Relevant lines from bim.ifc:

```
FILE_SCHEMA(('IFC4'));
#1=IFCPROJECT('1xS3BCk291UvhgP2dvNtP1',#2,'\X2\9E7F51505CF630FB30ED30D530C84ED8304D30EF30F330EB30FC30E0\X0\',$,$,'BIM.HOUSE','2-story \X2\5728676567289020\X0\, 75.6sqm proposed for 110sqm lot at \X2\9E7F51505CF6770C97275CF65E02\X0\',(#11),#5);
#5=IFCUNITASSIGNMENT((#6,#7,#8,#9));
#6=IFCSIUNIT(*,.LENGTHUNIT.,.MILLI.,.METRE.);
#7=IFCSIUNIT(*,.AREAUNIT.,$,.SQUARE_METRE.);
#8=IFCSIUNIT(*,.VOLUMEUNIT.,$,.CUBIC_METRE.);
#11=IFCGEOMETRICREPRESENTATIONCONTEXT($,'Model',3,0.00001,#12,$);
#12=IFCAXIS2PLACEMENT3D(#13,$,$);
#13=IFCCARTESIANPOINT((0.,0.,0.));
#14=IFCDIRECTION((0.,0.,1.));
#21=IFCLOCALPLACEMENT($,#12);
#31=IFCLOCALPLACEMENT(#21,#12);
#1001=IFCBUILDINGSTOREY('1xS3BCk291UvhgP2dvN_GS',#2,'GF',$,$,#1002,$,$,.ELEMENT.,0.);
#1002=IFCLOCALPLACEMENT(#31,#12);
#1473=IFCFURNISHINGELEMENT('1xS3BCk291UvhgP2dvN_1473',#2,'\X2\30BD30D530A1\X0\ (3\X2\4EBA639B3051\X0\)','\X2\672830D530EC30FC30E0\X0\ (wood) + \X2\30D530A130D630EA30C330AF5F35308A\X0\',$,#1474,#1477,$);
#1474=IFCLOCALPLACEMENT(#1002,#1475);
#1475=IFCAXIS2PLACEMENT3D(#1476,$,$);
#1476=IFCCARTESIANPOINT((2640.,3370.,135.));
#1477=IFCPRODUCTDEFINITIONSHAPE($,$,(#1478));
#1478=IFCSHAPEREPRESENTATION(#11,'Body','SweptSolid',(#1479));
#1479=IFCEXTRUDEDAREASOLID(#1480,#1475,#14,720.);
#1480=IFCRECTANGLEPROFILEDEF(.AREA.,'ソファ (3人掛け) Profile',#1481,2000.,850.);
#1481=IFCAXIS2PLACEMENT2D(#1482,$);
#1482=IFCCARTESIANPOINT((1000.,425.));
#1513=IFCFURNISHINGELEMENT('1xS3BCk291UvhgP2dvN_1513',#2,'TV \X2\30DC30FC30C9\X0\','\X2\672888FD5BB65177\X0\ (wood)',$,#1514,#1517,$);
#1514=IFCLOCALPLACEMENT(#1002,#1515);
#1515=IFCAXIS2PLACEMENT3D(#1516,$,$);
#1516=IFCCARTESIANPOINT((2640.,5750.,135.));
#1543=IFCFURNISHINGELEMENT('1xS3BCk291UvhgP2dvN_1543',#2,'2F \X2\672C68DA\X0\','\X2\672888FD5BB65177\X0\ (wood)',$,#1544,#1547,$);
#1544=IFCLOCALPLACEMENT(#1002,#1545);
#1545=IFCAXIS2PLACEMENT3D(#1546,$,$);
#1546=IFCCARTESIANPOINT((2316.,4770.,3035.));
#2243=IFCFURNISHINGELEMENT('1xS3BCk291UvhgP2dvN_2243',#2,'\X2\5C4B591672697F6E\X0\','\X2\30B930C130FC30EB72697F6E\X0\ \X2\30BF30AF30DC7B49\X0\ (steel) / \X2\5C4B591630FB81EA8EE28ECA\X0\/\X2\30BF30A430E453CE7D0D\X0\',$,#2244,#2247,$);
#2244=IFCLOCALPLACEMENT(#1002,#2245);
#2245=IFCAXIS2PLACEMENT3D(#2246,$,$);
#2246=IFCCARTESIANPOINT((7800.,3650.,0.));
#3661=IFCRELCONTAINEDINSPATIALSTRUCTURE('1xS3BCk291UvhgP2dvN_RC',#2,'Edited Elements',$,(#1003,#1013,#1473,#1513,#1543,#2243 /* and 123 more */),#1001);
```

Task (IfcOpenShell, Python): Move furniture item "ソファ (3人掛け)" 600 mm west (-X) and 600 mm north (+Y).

```python
import ifcopenshell
import ifcopenshell.api.geometry
import ifcopenshell.util.placement
import ifcopenshell.util.unit

model = ifcopenshell.open("bim.ifc")
unit_scale = ifcopenshell.util.unit.calculate_unit_scale(model)

item = model.by_guid("1xS3BCk291UvhgP2dvN_1473")
matrix = ifcopenshell.util.placement.get_local_placement(item.ObjectPlacement)
matrix[0, 3] -= 0.6 / unit_scale
matrix[1, 3] += 0.6 / unit_scale
ifcopenshell.api.geometry.edit_object_placement(model, product=item, matrix=matrix, is_si=False)

print(ifcopenshell.util.placement.get_local_placement(item.ObjectPlacement).round(3) + 0.0)

model.write("bim_edited.ifc")
```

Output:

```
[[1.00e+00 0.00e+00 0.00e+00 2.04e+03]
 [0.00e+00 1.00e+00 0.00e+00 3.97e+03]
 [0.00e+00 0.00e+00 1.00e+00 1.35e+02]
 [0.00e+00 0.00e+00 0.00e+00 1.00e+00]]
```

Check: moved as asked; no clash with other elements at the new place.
